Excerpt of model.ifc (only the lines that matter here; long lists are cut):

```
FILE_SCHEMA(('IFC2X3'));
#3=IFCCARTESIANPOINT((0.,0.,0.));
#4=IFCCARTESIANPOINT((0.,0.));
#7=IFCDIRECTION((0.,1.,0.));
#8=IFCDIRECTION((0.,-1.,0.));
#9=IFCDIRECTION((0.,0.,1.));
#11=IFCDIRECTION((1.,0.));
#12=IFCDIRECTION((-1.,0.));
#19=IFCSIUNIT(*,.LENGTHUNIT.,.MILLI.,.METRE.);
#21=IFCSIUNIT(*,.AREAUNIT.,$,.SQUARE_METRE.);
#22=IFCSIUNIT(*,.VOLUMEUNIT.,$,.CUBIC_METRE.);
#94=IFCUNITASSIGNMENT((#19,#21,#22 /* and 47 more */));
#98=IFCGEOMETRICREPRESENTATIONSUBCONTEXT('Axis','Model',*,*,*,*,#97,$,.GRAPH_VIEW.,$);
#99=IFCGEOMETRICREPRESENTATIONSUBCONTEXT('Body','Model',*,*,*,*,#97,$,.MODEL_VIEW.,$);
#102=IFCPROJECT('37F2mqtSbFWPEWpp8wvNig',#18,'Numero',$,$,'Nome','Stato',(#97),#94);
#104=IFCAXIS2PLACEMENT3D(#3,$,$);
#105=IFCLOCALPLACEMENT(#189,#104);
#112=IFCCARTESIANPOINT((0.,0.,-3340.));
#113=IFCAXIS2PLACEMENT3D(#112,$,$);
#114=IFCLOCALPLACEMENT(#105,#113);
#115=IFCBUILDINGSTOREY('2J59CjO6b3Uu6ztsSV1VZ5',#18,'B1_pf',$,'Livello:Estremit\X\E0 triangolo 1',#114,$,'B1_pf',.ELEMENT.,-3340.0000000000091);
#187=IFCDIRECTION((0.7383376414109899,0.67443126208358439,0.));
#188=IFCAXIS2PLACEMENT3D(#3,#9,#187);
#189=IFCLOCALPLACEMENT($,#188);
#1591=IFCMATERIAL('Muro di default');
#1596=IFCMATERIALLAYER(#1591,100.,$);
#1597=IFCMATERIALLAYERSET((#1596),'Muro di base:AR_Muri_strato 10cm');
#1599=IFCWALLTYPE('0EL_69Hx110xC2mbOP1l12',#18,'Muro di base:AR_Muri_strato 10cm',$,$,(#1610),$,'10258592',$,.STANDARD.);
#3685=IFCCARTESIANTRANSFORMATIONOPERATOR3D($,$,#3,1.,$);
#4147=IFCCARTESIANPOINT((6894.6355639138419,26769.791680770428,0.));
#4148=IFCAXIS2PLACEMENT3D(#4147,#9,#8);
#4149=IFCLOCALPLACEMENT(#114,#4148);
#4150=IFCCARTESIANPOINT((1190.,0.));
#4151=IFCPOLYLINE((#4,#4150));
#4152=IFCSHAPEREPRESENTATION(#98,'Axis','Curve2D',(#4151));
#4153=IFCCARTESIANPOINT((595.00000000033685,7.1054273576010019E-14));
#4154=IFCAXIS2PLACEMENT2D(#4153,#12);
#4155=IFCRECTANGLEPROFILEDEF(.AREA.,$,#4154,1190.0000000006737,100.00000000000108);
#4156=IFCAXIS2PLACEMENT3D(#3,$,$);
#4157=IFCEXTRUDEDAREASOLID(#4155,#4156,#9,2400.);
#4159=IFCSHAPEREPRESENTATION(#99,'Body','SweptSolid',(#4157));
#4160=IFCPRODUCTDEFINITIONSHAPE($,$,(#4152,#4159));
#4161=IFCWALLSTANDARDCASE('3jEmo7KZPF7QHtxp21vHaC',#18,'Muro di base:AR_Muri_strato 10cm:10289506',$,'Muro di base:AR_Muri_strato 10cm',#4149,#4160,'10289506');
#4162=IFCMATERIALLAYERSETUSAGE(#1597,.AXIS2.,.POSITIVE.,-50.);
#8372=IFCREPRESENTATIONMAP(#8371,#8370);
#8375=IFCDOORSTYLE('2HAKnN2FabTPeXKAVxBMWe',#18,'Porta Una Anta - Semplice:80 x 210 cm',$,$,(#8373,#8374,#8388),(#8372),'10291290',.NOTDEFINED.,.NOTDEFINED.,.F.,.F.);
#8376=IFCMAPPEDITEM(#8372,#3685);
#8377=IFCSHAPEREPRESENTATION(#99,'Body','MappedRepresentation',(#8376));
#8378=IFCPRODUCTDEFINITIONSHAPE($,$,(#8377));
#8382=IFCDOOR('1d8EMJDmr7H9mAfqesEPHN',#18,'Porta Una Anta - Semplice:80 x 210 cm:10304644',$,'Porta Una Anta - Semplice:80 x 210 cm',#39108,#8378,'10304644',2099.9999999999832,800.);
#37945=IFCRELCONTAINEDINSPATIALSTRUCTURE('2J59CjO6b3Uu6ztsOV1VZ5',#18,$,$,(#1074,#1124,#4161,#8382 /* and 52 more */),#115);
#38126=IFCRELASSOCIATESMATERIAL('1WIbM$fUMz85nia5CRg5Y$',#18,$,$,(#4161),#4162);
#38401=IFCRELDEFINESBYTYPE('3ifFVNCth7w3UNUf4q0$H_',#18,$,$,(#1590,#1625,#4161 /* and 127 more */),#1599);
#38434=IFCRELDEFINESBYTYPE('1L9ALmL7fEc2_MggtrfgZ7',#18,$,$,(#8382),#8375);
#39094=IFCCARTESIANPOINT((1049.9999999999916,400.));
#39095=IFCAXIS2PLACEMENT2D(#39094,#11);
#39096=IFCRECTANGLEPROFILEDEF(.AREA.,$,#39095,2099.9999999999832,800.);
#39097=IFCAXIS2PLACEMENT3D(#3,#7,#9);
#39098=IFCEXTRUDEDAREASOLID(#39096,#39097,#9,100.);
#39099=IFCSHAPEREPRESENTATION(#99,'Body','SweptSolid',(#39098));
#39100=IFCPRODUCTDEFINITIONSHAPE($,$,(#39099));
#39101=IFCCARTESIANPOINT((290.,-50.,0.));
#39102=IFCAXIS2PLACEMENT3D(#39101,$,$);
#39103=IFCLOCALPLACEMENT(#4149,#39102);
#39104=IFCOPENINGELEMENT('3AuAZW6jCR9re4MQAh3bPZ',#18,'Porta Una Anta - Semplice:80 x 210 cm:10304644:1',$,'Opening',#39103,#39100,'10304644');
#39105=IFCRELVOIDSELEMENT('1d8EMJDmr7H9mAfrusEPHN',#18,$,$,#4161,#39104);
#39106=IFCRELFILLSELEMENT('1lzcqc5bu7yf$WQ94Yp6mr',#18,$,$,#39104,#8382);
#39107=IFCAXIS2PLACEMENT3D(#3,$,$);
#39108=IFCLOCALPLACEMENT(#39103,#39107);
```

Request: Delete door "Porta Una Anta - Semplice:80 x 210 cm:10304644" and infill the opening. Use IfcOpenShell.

```python
import ifcopenshell
import ifcopenshell.api.feature
import ifcopenshell.api.root
import ifcopenshell.geom
import ifcopenshell.util.shape

model = ifcopenshell.open("model.ifc")
settings = ifcopenshell.geom.settings()


def volume(element):
    """Net volume in cubic metres, openings subtracted."""
    shape = ifcopenshell.geom.create_shape(settings, element)
    return ifcopenshell.util.shape.get_volume(shape.geometry)


door = model.by_guid("1d8EMJDmr7H9mAfqesEPHN")
opening = door.FillsVoids[0].RelatingOpeningElement
wall = opening.VoidsElements[0].RelatingBuildingElement
before = volume(wall)

ifcopenshell.api.root.remove_product(model, product=door)
ifcopenshell.api.feature.remove_feature(model, feature=opening)

after = volume(wall)

print(f"wall volume {before:.3f} -> {after:.3f} m3")

model.write("model_updated.ifc")
```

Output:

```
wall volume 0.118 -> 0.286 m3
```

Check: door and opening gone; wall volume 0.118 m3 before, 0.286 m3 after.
